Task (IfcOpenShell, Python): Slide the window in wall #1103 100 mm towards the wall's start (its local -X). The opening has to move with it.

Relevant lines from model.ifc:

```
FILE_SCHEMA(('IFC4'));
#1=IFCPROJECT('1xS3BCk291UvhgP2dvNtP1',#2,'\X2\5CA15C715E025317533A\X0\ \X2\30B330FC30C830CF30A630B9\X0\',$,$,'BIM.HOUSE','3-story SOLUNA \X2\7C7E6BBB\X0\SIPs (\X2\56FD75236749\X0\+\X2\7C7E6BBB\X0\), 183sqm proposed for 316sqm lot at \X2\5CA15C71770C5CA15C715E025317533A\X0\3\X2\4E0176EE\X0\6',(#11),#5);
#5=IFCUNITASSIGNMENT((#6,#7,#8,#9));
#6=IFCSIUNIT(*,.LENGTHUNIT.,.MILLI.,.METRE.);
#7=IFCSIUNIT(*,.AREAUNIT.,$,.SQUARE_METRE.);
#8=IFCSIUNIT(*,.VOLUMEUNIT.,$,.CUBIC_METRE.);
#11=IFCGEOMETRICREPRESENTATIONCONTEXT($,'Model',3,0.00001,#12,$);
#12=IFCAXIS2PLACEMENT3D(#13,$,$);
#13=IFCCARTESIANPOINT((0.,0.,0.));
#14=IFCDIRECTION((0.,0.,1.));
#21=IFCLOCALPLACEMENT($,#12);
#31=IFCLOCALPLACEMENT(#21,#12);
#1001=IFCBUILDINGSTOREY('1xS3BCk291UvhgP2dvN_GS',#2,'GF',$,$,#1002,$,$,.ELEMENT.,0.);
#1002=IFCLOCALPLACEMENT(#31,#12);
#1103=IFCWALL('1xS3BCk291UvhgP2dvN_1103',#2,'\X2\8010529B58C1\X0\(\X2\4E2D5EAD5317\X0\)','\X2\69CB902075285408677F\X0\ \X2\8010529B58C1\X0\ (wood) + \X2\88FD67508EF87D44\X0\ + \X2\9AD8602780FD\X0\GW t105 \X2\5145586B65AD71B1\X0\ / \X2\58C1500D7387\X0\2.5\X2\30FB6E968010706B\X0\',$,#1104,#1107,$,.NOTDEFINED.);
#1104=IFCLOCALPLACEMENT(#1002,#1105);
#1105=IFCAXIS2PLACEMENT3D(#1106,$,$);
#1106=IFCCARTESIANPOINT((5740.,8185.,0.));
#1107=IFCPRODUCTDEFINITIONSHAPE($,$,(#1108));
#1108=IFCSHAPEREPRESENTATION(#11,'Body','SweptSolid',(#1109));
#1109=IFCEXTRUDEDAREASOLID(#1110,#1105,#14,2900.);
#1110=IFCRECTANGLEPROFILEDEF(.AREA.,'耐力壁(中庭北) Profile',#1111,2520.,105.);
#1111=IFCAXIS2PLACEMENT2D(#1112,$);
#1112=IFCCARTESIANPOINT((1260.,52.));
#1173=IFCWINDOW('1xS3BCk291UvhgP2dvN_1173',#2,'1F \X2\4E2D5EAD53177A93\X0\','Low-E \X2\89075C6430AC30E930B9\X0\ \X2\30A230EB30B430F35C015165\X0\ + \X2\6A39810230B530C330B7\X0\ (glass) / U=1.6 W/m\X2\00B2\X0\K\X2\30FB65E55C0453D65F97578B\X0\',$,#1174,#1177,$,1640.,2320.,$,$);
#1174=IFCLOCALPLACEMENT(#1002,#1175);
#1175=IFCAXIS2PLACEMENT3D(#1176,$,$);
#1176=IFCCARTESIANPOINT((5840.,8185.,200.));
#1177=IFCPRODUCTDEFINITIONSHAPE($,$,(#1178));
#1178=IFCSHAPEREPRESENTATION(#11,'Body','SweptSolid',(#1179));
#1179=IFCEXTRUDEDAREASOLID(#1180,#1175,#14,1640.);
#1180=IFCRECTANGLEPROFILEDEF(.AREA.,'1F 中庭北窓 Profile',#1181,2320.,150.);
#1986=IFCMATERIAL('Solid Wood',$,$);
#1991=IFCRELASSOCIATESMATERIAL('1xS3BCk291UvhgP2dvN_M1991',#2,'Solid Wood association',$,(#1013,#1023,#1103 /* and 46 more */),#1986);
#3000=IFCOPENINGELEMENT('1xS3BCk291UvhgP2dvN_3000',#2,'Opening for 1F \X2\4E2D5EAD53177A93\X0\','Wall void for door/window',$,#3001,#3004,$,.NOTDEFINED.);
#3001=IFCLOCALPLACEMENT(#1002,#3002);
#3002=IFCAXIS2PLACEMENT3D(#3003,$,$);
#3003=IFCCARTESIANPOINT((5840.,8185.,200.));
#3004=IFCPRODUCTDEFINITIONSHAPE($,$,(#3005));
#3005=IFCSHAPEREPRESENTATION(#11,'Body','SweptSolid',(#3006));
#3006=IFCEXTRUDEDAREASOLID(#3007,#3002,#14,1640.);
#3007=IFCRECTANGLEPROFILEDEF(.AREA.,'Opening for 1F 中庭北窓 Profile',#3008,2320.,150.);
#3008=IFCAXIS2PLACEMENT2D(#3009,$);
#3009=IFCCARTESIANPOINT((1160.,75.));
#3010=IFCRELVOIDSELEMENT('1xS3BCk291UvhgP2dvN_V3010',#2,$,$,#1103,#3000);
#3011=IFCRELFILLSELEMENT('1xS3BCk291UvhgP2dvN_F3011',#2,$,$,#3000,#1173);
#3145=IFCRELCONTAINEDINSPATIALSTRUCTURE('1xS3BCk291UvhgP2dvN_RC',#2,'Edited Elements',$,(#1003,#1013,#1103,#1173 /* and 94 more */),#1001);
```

```python
import ifcopenshell
import ifcopenshell.api.geometry
import ifcopenshell.util.placement

model = ifcopenshell.open("model.ifc")

window = model.by_guid("1xS3BCk291UvhgP2dvN_1173")
opening = window.FillsVoids[0].RelatingOpeningElement
wall = opening.VoidsElements[0].RelatingBuildingElement

wall_matrix = ifcopenshell.util.placement.get_local_placement(wall.ObjectPlacement)
shift = wall_matrix[:3, 0] * -100.0
before = ifcopenshell.util.placement.get_local_placement(window.ObjectPlacement)[:3, 3].copy()

# The window is not placed relative to its opening, so move both.
for product in (opening, window):
    matrix = ifcopenshell.util.placement.get_local_placement(product.ObjectPlacement)
    matrix[:3, 3] += shift
    ifcopenshell.api.geometry.edit_object_placement(model, product=product, matrix=matrix, is_si=False)

after = ifcopenshell.util.placement.get_local_placement(window.ObjectPlacement)[:3, 3]
print("window moved by", (after - before).round(3) + 0.0)

model.write("model_updated.ifc")
```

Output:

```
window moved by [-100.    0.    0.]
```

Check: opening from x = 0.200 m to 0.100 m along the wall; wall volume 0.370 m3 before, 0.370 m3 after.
